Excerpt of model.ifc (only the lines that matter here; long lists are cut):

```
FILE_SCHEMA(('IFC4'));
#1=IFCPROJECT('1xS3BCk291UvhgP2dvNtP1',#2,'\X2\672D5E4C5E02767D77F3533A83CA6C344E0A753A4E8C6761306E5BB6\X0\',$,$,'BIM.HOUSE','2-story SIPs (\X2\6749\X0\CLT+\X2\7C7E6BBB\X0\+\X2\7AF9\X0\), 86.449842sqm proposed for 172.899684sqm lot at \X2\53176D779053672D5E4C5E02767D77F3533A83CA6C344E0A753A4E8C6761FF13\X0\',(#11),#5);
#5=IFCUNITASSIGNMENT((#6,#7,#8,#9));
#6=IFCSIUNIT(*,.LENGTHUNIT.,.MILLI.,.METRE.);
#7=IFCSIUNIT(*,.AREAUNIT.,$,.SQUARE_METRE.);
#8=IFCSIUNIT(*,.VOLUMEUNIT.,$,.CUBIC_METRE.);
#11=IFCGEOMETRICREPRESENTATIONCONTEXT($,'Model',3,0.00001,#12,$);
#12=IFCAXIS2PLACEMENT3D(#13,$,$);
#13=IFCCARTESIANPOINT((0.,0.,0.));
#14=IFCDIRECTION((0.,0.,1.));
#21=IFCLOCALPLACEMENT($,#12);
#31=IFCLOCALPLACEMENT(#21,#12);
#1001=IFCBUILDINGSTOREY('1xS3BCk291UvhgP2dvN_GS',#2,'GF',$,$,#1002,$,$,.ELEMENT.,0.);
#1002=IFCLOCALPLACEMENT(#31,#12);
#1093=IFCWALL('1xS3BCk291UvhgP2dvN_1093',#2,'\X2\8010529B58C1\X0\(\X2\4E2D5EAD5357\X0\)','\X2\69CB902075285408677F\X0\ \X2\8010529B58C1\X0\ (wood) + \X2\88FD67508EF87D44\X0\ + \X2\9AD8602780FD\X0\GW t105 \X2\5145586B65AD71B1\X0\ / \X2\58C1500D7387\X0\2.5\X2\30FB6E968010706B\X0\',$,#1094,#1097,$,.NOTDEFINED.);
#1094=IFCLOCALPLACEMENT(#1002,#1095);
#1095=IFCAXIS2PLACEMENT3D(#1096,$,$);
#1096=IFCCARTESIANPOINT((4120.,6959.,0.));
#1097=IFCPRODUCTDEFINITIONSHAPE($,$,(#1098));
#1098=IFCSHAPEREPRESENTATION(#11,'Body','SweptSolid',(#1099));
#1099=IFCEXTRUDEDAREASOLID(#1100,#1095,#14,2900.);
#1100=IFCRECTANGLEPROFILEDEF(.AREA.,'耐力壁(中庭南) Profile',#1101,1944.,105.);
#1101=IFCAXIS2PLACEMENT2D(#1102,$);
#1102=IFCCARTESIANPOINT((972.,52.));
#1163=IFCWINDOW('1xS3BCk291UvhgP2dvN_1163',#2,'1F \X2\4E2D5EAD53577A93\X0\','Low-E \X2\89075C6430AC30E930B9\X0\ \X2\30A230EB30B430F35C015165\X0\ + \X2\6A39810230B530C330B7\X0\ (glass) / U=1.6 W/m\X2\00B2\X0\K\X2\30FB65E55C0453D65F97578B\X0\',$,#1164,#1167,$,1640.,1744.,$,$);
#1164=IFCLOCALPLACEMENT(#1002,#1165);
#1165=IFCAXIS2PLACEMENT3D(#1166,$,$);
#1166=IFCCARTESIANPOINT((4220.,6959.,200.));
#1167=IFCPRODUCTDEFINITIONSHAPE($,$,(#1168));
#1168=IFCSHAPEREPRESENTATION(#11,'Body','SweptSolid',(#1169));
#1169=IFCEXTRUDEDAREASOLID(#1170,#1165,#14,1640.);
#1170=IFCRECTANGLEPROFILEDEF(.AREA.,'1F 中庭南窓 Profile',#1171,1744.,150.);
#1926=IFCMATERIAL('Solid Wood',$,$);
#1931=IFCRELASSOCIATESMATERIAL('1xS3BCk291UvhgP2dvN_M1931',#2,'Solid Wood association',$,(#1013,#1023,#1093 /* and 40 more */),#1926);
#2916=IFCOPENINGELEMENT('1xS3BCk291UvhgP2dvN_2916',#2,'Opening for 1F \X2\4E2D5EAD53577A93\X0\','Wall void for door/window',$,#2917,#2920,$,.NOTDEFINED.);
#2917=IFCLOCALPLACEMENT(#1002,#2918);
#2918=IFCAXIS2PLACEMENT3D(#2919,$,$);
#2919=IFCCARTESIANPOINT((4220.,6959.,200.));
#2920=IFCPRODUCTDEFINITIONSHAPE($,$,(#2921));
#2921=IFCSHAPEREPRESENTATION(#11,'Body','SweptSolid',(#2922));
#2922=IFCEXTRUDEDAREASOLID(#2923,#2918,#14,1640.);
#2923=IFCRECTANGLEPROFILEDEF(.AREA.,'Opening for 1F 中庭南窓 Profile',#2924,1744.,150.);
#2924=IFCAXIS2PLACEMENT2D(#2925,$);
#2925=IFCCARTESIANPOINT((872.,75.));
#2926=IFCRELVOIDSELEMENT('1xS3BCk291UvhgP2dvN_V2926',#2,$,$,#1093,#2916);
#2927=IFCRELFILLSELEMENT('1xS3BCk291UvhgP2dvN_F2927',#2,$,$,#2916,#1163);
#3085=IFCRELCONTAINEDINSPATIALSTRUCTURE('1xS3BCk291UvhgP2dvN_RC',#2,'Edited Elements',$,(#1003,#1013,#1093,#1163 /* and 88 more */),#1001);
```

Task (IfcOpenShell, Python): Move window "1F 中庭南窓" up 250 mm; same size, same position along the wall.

```python
import numpy as np
import ifcopenshell
import ifcopenshell.api.geometry
import ifcopenshell.util.placement
import ifcopenshell.util.unit

model = ifcopenshell.open("model.ifc")
unit_scale = ifcopenshell.util.unit.calculate_unit_scale(model)

window = model.by_id(1163)
opening = window.FillsVoids[0].RelatingOpeningElement
dz = 0.25 / unit_scale

shift = np.array([0.0, 0.0, dz])
# The window is not placed relative to its opening, so move both.
for product in (opening, window):
    matrix = ifcopenshell.util.placement.get_local_placement(product.ObjectPlacement)
    matrix[:3, 3] += shift
    ifcopenshell.api.geometry.edit_object_placement(model, product=product, matrix=matrix, is_si=False)

print(f"moved by {dz * unit_scale:+.3f} m")

model.write("model_updated.ifc")
```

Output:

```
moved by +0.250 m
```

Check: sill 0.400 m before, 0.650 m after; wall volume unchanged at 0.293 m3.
